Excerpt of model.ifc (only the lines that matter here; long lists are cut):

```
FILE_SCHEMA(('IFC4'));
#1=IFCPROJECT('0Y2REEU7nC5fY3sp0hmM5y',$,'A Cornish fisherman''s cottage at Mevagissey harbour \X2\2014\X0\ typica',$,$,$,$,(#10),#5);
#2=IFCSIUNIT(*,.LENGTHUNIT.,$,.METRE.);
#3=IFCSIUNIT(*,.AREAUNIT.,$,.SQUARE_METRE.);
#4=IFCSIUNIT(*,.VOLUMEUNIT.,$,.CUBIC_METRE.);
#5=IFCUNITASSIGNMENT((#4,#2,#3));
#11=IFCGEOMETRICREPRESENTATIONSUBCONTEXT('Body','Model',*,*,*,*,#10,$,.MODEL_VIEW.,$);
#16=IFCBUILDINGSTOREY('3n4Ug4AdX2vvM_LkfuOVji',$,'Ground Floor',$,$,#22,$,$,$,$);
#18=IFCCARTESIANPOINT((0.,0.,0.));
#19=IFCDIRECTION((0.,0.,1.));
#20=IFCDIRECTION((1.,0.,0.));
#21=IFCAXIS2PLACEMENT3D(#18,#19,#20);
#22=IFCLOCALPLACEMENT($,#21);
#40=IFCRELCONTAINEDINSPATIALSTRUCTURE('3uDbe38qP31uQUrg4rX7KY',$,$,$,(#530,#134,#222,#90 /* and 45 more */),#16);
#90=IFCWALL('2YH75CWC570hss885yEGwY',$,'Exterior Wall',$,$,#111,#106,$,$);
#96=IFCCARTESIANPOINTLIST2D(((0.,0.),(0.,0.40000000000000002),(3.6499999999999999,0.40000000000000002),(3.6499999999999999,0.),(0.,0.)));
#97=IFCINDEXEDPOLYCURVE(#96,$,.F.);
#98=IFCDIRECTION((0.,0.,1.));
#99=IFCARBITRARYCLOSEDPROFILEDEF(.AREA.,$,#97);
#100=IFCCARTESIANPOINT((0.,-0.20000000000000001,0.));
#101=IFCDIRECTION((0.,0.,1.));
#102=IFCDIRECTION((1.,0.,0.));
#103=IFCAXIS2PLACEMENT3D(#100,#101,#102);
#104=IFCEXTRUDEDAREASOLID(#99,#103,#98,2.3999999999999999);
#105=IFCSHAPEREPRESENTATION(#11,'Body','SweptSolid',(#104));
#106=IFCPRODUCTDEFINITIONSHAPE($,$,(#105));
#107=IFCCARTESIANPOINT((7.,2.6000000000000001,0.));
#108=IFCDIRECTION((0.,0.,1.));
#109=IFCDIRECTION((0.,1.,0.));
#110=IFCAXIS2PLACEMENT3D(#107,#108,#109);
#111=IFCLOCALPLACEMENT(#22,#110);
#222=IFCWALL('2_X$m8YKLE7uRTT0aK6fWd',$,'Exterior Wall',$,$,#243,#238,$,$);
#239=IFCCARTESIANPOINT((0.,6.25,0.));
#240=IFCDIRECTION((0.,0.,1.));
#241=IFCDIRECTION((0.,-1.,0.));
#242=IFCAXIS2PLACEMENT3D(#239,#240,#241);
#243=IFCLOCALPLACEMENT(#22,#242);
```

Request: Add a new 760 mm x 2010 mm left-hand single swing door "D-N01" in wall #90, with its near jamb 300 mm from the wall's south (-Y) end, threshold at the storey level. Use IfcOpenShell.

```python
import numpy as np
import ifcopenshell
import ifcopenshell.api.feature
import ifcopenshell.api.geometry
import ifcopenshell.api.root
import ifcopenshell.api.spatial
import ifcopenshell.geom
import ifcopenshell.util.element
import ifcopenshell.util.placement
import ifcopenshell.util.representation
import ifcopenshell.util.shape
import ifcopenshell.util.unit

model = ifcopenshell.open("model.ifc")
unit_scale = ifcopenshell.util.unit.calculate_unit_scale(model)
settings = ifcopenshell.geom.settings()


def volume(element):
    """Net volume in cubic metres, openings subtracted."""
    shape = ifcopenshell.geom.create_shape(settings, element)
    return ifcopenshell.util.shape.get_volume(shape.geometry)


wall = model.by_guid("2YH75CWC570hss885yEGwY")
storey = ifcopenshell.util.element.get_container(wall, ifc_class="IfcBuildingStorey")
context = ifcopenshell.util.representation.get_context(model, "Model", "Body", "MODEL_VIEW")
before = volume(wall)

width, height, from_end, sill = 0.76, 2.01, 0.3, 0.0  # metres

# The wall runs along its own X axis, and the end named is its -X end.
wall_shape = ifcopenshell.geom.create_shape(settings, wall)
x, y, z = ifcopenshell.util.shape.get_vertices(wall_shape.geometry).T
start = x.min() + from_end
face, thickness = float(y.min()), float(y.max() - y.min())
wall_matrix = ifcopenshell.util.placement.get_local_placement(wall.ObjectPlacement)
level = ifcopenshell.util.placement.get_local_placement(storey.ObjectPlacement)[2, 3]


def in_wall(x, y):
    """Placement at x, y metres in the wall's axes, at sill height."""
    matrix = wall_matrix.copy()
    matrix[:, 3] = wall_matrix @ np.array([x / unit_scale, y / unit_scale, 0.0, 1.0])
    matrix[2, 3] = level + sill / unit_scale
    return matrix


# Opening: a box that overshoots both wall faces by 50 mm.
opening = ifcopenshell.api.root.create_entity(model, ifc_class="IfcOpeningElement", predefined_type="OPENING")
box = ifcopenshell.api.geometry.add_wall_representation(
    model, context=context, length=width, height=height, thickness=thickness + 0.1
)
ifcopenshell.api.geometry.assign_representation(model, product=opening, representation=box)
ifcopenshell.api.geometry.edit_object_placement(model, product=opening, matrix=in_wall(start, face - 0.05), is_si=False)
ifcopenshell.api.feature.add_feature(model, feature=opening, element=wall)

door = ifcopenshell.api.root.create_entity(model, ifc_class="IfcDoor", name="D-N01", predefined_type="DOOR")
door.OverallWidth, door.OverallHeight = width / unit_scale, height / unit_scale
door.OperationType = "SINGLE_SWING_LEFT"
body = ifcopenshell.api.geometry.add_door_representation(
    model,
    context=context,
    overall_width=door.OverallWidth,
    overall_height=door.OverallHeight,
    operation_type="SINGLE_SWING_LEFT",
    lining_properties={"LiningDepth": thickness / unit_scale, "ThresholdDepth": thickness / unit_scale},
)
ifcopenshell.api.geometry.assign_representation(model, product=door, representation=body)
ifcopenshell.api.spatial.assign_container(model, products=[door], relating_structure=storey)
ifcopenshell.api.feature.add_filling(model, opening=opening, element=door)

# The lining spans the wall, so the door starts at the wall face.
ifcopenshell.api.geometry.edit_object_placement(model, product=door, matrix=in_wall(start, face), is_si=False)

after = volume(wall)

print(f"wall volume {before:.3f} -> {after:.3f} m3")

model.write("model_edited.ifc")
```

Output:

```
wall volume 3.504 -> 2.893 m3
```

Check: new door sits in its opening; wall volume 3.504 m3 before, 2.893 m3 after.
